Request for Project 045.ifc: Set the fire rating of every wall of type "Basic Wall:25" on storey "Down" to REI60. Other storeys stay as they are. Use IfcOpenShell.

First a look at what the model holds.

```python
import ifcopenshell
import ifcopenshell.util.element

model = ifcopenshell.open("Project 045.ifc")
print(model.schema)
storey = next(s for s in model.by_type("IfcBuildingStorey") if s.Name == "Down")
walls = [e for e in ifcopenshell.util.element.get_decomposition(storey) if e.is_a("IfcWall")]
seen = {}
for e in walls:
    element_type = ifcopenshell.util.element.get_type(e)
    key = (element_type.Name if element_type != e and element_type else None, ifcopenshell.util.element.get_pset(e, "Pset_WallCommon", "FireRating"))
    seen[key] = seen.get(key, 0) + 1
for (name, value), count in sorted(seen.items(), key=str):
    print(count, "x", name, "|", value)
```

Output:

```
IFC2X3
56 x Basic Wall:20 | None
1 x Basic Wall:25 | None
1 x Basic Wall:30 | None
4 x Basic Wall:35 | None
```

```python
import ifcopenshell
import ifcopenshell.api.pset
import ifcopenshell.util.element

model = ifcopenshell.open("Project 045.ifc")

storey = next(s for s in model.by_type("IfcBuildingStorey") if s.Name == "Down")
walls = [e for e in ifcopenshell.util.element.get_decomposition(storey) if e.is_a("IfcWall")]

count = 0
for e in walls:
    element_type = ifcopenshell.util.element.get_type(e)
    if element_type in (None, e) or element_type.Name != "Basic Wall:25":
        continue
    # add_pset returns the element's existing set when there is one.
    pset = ifcopenshell.api.pset.add_pset(model, product=e, name="Pset_WallCommon")
    ifcopenshell.api.pset.edit_pset(model, pset=pset, properties={"FireRating": "REI60"})
    count += 1

print(count, "walls updated")

model.write("Project 045-out.ifc")
```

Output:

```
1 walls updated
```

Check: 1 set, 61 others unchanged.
